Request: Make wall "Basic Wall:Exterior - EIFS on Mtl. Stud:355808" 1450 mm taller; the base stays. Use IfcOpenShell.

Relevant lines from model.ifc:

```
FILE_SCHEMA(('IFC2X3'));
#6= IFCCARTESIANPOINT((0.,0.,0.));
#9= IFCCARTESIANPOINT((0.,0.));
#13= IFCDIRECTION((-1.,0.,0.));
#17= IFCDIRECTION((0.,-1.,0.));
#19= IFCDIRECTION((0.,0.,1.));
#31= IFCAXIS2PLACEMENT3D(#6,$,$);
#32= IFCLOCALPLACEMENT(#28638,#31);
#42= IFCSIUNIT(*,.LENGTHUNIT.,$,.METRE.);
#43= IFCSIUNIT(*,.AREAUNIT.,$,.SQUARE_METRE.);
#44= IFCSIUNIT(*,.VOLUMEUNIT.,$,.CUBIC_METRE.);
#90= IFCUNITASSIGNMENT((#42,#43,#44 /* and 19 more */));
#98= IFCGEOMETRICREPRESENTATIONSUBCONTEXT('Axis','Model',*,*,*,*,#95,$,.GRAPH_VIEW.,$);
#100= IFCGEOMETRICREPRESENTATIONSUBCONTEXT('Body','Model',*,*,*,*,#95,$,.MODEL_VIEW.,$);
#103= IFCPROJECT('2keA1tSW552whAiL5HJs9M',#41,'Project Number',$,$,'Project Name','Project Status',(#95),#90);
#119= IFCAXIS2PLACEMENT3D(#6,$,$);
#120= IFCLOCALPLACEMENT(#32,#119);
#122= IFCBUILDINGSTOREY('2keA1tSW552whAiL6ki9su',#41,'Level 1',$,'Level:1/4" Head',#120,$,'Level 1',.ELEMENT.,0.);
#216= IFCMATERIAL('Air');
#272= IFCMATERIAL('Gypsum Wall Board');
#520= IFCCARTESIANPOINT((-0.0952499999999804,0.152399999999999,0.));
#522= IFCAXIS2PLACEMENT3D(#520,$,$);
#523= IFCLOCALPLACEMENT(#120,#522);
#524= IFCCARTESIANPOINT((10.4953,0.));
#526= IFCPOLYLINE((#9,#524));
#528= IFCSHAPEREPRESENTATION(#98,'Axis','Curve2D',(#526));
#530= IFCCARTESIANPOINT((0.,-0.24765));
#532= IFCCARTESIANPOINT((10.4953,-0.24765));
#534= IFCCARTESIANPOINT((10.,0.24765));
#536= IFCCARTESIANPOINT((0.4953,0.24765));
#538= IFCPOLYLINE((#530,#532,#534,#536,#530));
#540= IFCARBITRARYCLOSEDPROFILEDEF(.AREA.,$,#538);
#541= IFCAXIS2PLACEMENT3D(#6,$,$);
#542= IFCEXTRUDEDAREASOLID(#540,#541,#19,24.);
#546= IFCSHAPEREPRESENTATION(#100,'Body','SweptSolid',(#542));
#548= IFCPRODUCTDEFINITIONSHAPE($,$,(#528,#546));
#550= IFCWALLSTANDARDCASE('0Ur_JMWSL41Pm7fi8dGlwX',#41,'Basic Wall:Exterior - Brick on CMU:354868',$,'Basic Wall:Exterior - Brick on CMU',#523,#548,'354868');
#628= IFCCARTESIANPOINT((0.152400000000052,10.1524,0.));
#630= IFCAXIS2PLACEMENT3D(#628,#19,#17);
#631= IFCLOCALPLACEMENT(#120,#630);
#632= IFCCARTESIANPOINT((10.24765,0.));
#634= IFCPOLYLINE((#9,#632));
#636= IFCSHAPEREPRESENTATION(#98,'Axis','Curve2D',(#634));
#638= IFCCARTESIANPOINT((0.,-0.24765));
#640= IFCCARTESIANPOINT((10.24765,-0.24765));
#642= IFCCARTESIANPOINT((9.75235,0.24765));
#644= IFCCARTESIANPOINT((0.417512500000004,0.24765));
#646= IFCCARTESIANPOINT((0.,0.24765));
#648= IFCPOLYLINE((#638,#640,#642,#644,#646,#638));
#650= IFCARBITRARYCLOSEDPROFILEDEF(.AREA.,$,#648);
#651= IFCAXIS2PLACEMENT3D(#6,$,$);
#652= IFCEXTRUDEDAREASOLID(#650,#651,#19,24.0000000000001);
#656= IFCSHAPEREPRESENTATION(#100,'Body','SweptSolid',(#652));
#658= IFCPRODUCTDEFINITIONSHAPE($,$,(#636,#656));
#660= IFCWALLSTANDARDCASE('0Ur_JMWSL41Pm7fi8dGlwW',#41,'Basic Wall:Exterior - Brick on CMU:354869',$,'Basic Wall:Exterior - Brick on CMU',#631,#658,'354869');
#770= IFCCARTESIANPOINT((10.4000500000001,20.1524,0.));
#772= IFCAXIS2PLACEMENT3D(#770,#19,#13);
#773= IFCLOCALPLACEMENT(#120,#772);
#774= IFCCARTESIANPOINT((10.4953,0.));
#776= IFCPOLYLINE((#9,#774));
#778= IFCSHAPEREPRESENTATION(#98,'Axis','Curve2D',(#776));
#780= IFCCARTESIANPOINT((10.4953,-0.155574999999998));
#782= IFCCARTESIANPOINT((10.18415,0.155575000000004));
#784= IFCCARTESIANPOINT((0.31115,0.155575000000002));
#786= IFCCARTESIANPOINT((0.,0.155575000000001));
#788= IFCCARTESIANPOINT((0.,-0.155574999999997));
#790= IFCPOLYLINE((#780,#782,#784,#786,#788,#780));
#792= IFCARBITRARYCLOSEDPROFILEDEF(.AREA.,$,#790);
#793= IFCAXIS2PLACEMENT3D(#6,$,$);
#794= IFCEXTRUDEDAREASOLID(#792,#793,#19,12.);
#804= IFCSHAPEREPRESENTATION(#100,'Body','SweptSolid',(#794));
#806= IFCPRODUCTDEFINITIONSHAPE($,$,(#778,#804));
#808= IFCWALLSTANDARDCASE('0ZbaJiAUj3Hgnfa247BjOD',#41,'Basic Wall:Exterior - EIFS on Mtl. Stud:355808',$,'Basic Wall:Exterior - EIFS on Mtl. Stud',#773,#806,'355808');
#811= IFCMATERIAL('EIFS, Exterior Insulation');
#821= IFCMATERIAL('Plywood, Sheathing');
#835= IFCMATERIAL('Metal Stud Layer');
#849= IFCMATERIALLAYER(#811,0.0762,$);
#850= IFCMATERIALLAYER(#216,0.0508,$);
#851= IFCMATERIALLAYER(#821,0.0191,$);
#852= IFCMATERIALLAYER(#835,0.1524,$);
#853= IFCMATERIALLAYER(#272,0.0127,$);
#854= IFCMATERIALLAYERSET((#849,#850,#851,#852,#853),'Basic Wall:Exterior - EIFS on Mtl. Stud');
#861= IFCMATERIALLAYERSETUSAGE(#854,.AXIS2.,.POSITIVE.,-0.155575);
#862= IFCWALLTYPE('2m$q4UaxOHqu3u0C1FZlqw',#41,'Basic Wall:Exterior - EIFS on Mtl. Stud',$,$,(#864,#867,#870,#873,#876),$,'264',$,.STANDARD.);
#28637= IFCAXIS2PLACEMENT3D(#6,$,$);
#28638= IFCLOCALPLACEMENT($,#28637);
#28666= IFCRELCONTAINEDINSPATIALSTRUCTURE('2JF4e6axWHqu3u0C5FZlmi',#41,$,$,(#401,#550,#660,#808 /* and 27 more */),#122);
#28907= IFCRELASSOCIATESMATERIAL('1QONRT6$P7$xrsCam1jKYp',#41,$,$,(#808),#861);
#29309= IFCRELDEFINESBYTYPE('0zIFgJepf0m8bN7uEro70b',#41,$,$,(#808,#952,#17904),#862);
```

```python
import ifcopenshell
import ifcopenshell.geom
import ifcopenshell.util.representation
import ifcopenshell.util.shape
import ifcopenshell.util.unit

model = ifcopenshell.open("model.ifc")
unit_scale = ifcopenshell.util.unit.calculate_unit_scale(model)
settings = ifcopenshell.geom.settings()


def volume(element):
    """Net volume in cubic metres, openings subtracted."""
    shape = ifcopenshell.geom.create_shape(settings, element)
    return ifcopenshell.util.shape.get_volume(shape.geometry)


wall = model.by_id(808)
before = volume(wall)

body = ifcopenshell.util.representation.get_representation(wall, "Model", "Body")
solid = body.Items[0]
old_height = solid.Depth
solid.Depth += 1.45 / unit_scale
after = volume(wall)

print(f"height {old_height:g} -> {solid.Depth:g}, volume {before:.3f} -> {after:.3f} m3")

model.write("model_updated.ifc")
```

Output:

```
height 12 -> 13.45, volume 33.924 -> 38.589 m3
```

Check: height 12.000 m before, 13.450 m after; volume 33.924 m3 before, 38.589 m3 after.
